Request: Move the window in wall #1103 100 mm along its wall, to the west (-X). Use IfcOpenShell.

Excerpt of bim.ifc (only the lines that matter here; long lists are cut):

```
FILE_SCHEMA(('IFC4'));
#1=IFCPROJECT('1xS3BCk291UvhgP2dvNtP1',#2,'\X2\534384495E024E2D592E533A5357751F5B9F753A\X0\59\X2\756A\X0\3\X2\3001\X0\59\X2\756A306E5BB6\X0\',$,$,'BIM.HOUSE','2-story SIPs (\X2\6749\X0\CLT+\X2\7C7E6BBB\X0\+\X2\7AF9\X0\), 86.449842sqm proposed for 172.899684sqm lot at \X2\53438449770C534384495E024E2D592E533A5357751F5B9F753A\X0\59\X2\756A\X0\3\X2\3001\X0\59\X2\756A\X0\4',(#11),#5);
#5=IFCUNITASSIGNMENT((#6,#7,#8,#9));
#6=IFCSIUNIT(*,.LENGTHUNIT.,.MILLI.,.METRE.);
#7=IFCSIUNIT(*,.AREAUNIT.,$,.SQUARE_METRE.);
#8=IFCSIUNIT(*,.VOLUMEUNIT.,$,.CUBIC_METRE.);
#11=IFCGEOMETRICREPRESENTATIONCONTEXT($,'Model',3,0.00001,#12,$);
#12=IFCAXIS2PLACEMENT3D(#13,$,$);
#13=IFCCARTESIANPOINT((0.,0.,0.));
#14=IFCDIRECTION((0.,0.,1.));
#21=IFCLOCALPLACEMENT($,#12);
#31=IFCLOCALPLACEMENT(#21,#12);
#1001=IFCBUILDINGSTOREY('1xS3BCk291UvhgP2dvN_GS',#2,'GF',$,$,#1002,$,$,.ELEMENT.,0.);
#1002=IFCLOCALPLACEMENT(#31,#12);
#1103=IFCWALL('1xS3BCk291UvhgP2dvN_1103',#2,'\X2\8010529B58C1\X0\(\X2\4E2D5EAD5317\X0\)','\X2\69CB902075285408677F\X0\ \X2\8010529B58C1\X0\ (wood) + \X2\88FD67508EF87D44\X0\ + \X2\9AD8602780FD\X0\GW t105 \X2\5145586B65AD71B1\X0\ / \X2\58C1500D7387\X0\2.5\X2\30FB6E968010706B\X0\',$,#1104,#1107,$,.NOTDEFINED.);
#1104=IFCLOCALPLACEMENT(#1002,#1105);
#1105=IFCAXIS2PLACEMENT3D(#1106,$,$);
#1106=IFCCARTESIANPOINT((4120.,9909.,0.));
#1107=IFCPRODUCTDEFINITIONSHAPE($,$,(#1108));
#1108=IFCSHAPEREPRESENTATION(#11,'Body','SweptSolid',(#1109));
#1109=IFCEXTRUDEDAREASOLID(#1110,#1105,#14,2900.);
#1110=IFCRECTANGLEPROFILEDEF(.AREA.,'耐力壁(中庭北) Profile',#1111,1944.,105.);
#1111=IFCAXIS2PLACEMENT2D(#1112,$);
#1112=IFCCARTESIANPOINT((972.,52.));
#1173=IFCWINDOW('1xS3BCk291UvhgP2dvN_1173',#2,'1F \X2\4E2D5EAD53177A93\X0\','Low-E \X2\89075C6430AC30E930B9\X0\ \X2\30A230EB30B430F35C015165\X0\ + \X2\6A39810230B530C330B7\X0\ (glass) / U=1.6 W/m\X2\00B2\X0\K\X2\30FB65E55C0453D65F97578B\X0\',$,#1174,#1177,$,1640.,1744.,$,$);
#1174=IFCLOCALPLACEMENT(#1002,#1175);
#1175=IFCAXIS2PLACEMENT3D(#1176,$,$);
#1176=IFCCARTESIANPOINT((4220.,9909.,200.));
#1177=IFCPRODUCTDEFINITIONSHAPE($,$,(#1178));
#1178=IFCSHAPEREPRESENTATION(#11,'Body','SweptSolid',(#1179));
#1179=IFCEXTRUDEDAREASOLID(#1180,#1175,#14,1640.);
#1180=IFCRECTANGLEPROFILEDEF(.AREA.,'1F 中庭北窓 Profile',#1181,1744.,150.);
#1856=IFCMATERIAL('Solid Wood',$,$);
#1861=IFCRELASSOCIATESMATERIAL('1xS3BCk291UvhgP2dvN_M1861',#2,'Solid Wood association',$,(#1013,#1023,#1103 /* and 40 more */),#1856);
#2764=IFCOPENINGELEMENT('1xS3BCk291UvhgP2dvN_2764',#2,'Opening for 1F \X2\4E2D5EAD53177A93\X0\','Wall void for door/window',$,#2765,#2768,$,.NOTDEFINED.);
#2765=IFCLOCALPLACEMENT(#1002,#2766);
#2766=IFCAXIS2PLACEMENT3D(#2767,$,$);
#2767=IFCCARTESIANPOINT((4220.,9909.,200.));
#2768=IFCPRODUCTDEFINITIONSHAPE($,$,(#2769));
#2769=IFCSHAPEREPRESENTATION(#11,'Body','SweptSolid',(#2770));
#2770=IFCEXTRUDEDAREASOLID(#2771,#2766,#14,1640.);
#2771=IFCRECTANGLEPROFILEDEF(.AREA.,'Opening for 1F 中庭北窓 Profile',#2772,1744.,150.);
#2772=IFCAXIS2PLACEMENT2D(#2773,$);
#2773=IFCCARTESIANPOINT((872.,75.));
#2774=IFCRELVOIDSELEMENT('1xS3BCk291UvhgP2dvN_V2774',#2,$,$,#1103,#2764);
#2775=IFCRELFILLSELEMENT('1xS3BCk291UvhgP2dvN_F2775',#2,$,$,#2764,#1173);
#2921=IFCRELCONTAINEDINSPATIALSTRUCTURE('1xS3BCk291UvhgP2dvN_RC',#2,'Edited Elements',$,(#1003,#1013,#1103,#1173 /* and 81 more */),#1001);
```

```python
import ifcopenshell
import ifcopenshell.api.geometry
import ifcopenshell.util.placement

model = ifcopenshell.open("bim.ifc")

window = model.by_guid("1xS3BCk291UvhgP2dvN_1173")
opening = window.FillsVoids[0].RelatingOpeningElement
wall = opening.VoidsElements[0].RelatingBuildingElement

wall_matrix = ifcopenshell.util.placement.get_local_placement(wall.ObjectPlacement)
shift = wall_matrix[:3, 0] * -100.0
before = ifcopenshell.util.placement.get_local_placement(window.ObjectPlacement)[:3, 3].copy()

# The window is not placed relative to its opening, so move both.
for product in (opening, window):
    matrix = ifcopenshell.util.placement.get_local_placement(product.ObjectPlacement)
    matrix[:3, 3] += shift
    ifcopenshell.api.geometry.edit_object_placement(model, product=product, matrix=matrix, is_si=False)

after = ifcopenshell.util.placement.get_local_placement(window.ObjectPlacement)[:3, 3]
print("window moved by", (after - before).round(3) + 0.0)

model.write("bim-out.ifc")
```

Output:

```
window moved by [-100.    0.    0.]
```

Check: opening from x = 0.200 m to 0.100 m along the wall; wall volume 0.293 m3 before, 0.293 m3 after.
